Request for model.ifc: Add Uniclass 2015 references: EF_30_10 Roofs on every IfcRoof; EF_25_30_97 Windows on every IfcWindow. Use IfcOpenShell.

First a look at what the model holds.

```python
import ifcopenshell

model = ifcopenshell.open("model.ifc")
print(model.schema)
print("classifications:", [c.Name for c in model.by_type("IfcClassification")])
for ifc_class in ("IfcDoor", "IfcRoof", "IfcStair", "IfcWall", "IfcWindow"):
    print(ifc_class, len(model.by_type(ifc_class)))
```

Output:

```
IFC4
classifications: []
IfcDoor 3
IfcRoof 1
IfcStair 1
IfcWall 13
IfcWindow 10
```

```python
import ifcopenshell
import ifcopenshell.api.classification

model = ifcopenshell.open("model.ifc")

system = ifcopenshell.api.classification.add_classification(model, classification="Uniclass 2015")

codes = {
    "IfcRoof": ("EF_30_10", "Roofs"),
    "IfcWindow": ("EF_25_30_97", "Windows"),
}
for ifc_class, (code, name) in codes.items():
    products = model.by_type(ifc_class)
    ifcopenshell.api.classification.add_reference(
        model, products=products, classification=system, identification=code, name=name
    )
    print(code, len(products))

model.write("model_edited.ifc")
```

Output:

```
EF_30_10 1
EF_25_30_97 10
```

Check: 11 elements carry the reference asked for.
